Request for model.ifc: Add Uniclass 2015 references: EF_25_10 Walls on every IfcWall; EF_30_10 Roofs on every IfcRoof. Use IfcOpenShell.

First a look at what the model holds.

```python
import ifcopenshell

model = ifcopenshell.open("model.ifc")
print(model.schema)
print("classifications:", [c.Name for c in model.by_type("IfcClassification")])
for ifc_class in ("IfcDoor", "IfcRoof", "IfcStair", "IfcWall", "IfcWindow"):
    print(ifc_class, len(model.by_type(ifc_class)))
```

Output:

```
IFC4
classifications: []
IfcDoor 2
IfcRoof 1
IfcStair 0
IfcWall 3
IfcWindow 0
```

```python
import ifcopenshell
import ifcopenshell.api.classification

model = ifcopenshell.open("model.ifc")

system = ifcopenshell.api.classification.add_classification(model, classification="Uniclass 2015")

codes = {
    "IfcWall": ("EF_25_10", "Walls"),
    "IfcRoof": ("EF_30_10", "Roofs"),
}
for ifc_class, (code, name) in codes.items():
    products = model.by_type(ifc_class)
    ifcopenshell.api.classification.add_reference(
        model, products=products, classification=system, identification=code, name=name
    )
    print(code, len(products))

model.write("model-out.ifc")
```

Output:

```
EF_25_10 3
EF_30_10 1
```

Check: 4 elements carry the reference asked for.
